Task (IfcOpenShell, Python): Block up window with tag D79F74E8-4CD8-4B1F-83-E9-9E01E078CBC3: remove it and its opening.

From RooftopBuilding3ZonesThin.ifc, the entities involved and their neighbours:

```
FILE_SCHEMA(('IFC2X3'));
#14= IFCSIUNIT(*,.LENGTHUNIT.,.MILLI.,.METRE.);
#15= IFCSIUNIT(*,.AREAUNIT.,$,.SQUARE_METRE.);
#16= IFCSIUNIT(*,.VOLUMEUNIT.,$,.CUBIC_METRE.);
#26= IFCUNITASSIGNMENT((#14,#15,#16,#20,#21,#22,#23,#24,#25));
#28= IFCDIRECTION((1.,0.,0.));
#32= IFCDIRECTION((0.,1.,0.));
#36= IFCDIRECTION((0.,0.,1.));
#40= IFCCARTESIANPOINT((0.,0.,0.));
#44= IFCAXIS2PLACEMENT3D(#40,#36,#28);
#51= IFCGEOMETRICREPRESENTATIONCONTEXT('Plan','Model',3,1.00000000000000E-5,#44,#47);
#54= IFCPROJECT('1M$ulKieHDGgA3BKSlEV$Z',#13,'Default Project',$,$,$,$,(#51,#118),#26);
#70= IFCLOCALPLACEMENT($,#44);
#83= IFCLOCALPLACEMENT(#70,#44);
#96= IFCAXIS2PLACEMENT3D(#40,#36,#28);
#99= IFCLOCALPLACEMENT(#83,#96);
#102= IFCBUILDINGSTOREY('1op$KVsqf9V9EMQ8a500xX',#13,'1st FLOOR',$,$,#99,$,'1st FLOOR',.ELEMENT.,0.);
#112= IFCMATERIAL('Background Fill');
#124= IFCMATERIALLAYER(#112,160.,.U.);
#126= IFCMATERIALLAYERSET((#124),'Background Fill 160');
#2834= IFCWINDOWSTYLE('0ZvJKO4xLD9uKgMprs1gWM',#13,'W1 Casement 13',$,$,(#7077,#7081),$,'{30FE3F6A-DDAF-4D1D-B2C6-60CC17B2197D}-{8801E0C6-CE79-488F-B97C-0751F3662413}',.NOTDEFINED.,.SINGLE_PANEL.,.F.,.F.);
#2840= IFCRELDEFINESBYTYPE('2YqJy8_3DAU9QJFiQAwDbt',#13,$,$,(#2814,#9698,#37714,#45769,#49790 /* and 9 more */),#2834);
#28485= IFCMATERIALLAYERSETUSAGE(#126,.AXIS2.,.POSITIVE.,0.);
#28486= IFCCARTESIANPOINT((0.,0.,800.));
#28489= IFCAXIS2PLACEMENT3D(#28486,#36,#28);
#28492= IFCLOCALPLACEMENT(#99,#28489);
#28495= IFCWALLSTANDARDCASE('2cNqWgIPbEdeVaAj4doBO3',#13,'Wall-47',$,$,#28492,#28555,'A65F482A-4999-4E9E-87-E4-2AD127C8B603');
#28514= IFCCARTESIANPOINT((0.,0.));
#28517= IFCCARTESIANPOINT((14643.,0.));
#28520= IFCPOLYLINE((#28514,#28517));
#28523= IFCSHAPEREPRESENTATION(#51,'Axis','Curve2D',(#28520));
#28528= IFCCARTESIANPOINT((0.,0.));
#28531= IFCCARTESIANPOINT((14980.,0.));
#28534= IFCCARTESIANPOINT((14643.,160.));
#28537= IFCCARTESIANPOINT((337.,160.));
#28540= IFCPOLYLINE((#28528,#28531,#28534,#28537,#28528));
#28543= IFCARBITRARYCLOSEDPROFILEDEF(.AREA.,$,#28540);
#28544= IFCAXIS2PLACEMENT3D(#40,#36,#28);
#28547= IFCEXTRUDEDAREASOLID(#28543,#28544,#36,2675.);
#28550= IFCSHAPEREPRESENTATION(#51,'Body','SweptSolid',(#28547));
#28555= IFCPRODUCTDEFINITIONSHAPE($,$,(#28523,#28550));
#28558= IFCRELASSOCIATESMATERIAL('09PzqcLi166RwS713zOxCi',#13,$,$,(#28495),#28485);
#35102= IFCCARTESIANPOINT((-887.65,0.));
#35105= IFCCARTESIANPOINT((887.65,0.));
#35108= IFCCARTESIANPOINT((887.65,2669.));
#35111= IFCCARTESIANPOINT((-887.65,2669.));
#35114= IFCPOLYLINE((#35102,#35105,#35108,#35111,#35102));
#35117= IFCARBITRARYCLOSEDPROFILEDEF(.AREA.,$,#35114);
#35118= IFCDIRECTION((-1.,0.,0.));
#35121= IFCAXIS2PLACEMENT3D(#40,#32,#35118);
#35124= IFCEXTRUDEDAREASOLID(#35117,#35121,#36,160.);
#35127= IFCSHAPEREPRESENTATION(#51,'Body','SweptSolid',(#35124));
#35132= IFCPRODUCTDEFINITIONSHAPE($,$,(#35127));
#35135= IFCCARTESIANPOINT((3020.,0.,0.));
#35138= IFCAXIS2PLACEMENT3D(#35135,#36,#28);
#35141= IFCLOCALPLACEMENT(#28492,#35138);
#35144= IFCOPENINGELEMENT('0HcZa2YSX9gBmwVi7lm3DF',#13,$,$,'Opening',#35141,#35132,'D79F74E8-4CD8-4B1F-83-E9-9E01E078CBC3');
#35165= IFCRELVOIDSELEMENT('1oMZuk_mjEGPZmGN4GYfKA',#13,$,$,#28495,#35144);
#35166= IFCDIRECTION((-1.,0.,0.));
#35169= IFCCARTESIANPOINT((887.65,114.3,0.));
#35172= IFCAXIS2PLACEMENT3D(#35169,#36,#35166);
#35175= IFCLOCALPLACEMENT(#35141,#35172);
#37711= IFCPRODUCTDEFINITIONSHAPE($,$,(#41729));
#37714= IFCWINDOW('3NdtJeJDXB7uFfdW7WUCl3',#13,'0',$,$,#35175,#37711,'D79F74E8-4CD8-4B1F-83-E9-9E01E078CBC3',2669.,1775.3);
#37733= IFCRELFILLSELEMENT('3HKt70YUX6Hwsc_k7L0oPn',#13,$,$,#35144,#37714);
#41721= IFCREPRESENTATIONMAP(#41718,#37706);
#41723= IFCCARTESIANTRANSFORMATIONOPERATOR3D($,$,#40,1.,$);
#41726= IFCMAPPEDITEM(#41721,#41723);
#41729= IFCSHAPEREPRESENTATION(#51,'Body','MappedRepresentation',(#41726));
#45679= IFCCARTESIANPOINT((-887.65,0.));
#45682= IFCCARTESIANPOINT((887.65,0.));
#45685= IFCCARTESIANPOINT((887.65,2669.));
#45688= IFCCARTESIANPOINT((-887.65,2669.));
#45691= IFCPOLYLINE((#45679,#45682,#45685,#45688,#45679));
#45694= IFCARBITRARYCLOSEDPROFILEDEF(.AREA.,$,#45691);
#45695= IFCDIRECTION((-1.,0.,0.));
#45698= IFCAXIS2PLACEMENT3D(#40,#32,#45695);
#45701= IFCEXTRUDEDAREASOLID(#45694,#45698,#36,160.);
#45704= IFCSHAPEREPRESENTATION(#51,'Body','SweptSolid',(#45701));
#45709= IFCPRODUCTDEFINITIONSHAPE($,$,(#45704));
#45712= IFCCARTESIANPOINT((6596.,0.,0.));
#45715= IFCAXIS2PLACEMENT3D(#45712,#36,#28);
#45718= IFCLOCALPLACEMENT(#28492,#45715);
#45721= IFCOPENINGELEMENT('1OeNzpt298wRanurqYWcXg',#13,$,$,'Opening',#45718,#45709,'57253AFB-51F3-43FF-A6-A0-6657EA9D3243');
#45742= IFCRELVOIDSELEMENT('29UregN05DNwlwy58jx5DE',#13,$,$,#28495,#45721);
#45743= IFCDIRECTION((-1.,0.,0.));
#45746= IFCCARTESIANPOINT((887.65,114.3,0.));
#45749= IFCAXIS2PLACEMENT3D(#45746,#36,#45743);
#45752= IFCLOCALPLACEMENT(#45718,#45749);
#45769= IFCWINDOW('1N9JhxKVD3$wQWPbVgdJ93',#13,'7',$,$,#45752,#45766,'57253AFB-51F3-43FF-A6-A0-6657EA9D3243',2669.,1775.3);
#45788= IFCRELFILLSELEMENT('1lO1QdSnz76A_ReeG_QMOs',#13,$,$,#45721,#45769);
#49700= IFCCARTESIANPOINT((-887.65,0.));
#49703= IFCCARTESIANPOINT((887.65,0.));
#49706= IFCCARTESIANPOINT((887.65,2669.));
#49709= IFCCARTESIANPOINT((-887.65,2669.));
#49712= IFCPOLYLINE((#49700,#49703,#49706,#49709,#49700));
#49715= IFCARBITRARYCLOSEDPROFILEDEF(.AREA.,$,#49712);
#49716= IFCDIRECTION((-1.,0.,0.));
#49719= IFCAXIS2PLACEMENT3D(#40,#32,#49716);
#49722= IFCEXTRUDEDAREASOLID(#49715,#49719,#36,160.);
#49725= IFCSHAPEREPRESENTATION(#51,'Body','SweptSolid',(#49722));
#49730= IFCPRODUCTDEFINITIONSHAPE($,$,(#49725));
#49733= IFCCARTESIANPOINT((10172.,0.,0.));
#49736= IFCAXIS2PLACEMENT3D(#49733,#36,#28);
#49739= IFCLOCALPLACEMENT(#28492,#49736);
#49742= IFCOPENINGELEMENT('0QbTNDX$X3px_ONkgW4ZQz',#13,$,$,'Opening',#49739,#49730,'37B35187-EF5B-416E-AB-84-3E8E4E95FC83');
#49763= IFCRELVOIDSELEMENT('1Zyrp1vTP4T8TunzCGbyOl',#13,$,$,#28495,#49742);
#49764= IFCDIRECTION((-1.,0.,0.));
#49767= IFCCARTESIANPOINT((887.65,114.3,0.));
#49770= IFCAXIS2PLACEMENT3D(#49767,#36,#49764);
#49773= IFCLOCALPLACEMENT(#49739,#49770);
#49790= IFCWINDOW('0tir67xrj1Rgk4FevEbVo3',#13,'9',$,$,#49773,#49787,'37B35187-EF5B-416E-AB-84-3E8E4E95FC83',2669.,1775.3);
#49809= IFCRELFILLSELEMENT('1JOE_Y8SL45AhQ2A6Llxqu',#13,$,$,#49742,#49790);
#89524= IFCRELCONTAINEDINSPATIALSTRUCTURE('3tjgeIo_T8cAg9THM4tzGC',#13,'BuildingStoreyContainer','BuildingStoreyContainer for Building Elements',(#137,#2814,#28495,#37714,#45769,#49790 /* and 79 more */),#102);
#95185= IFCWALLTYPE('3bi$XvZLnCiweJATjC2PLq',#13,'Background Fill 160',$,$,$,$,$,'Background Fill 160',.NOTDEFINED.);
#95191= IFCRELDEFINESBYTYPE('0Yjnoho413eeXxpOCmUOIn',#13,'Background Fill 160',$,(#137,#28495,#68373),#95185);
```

```python
import ifcopenshell
import ifcopenshell.api.feature
import ifcopenshell.api.root
import ifcopenshell.geom
import ifcopenshell.util.shape

model = ifcopenshell.open("RooftopBuilding3ZonesThin.ifc")
settings = ifcopenshell.geom.settings()


def volume(element):
    """Net volume in cubic metres, openings subtracted."""
    shape = ifcopenshell.geom.create_shape(settings, element)
    return ifcopenshell.util.shape.get_volume(shape.geometry)


window = model.by_id(37714)
opening = window.FillsVoids[0].RelatingOpeningElement
wall = opening.VoidsElements[0].RelatingBuildingElement
before = volume(wall)

ifcopenshell.api.root.remove_product(model, product=window)
ifcopenshell.api.feature.remove_feature(model, feature=opening)

after = volume(wall)

print(f"wall volume {before:.3f} -> {after:.3f} m3")

model.write("RooftopBuilding3ZonesThin_updated.ifc")
```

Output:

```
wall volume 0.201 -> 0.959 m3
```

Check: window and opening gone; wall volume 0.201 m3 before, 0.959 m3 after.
